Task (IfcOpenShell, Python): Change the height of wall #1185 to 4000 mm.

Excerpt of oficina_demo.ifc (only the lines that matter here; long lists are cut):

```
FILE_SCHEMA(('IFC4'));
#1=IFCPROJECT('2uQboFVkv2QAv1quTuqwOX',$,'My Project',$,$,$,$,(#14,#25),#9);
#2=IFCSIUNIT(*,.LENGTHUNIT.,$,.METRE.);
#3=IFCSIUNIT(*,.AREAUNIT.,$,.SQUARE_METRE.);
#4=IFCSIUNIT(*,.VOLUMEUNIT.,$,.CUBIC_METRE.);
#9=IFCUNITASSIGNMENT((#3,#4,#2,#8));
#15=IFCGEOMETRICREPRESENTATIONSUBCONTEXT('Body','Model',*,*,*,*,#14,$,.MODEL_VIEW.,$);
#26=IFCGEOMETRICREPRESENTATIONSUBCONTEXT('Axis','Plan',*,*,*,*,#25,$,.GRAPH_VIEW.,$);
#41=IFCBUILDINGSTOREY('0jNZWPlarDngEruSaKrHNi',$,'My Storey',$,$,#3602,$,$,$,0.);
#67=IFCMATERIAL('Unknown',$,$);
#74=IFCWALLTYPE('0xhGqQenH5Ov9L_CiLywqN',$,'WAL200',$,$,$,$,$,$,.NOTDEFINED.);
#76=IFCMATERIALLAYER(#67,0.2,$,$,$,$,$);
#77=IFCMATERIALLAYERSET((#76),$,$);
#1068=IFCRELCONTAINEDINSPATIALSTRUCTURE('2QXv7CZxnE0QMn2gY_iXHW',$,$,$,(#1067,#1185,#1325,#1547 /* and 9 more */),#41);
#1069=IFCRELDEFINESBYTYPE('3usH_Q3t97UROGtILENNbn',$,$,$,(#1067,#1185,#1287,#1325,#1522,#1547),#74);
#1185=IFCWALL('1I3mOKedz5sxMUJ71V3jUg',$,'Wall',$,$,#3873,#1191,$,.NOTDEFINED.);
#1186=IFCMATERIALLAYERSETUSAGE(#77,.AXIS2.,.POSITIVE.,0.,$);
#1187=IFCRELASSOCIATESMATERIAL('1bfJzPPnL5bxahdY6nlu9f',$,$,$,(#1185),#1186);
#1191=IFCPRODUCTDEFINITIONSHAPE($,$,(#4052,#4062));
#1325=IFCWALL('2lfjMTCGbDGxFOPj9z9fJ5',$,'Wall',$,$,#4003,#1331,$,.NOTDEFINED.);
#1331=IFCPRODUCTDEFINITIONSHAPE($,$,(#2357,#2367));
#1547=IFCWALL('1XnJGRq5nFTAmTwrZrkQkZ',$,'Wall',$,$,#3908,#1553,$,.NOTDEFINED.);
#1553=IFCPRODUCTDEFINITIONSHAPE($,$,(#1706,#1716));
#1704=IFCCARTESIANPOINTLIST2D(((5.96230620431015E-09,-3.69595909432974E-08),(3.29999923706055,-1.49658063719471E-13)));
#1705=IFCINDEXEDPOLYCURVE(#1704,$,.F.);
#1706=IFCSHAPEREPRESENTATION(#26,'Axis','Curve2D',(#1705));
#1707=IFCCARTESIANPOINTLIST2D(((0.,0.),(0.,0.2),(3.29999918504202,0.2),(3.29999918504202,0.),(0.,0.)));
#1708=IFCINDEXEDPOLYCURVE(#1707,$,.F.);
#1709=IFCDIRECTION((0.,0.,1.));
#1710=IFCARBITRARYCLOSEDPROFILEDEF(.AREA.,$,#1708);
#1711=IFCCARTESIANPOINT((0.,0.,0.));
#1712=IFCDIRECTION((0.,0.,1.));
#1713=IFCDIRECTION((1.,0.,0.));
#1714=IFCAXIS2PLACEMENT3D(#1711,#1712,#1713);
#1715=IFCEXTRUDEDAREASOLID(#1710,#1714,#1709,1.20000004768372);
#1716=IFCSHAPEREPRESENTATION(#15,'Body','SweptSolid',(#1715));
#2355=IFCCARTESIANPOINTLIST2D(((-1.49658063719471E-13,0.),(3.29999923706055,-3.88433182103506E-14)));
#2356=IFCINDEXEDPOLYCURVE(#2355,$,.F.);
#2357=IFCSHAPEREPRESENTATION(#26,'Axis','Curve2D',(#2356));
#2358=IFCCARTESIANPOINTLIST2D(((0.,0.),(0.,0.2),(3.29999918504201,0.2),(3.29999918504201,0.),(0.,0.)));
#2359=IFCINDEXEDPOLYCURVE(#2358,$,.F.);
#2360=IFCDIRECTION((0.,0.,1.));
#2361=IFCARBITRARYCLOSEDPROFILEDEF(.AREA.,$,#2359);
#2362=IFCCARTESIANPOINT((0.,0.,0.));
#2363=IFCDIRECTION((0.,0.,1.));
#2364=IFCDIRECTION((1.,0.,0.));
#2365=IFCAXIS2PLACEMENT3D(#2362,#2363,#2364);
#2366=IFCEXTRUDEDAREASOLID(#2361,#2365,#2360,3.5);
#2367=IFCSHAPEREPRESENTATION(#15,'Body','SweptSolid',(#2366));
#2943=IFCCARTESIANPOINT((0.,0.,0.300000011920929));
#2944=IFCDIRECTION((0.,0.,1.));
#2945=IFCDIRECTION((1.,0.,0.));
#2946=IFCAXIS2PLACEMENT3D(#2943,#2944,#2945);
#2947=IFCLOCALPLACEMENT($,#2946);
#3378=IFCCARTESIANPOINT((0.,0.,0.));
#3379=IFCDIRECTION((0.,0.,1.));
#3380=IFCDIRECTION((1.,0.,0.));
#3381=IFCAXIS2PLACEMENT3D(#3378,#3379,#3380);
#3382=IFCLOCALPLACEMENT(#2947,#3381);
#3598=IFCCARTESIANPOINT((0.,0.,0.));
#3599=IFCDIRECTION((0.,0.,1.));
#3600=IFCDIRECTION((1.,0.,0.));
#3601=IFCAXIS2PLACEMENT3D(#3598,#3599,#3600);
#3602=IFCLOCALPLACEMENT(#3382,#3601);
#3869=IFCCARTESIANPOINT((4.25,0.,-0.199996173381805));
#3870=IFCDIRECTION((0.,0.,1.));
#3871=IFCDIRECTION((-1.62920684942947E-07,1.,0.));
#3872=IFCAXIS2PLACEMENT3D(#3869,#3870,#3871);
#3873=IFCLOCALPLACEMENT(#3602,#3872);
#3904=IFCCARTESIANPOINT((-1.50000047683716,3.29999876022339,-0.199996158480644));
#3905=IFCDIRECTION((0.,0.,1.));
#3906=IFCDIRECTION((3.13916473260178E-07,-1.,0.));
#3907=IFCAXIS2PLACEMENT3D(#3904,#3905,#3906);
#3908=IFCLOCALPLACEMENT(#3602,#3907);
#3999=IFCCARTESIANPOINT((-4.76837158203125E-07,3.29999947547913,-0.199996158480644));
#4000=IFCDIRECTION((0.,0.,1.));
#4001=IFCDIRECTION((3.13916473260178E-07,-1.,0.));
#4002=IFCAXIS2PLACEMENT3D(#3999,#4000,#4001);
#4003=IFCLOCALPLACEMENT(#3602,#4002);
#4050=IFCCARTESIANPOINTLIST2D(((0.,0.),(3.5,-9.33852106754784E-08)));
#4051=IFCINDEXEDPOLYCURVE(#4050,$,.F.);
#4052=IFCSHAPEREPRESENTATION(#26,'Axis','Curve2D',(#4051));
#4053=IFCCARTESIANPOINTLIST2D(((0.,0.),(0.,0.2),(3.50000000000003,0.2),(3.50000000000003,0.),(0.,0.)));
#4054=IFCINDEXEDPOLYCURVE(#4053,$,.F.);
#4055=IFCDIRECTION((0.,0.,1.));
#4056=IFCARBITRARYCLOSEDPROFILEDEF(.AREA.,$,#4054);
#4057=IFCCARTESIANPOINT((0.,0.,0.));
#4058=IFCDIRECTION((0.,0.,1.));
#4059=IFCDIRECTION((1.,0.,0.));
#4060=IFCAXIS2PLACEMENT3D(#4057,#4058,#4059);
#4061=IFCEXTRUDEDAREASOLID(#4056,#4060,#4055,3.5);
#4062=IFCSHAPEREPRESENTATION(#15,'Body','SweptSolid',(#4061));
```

```python
import ifcopenshell
import ifcopenshell.geom
import ifcopenshell.util.representation
import ifcopenshell.util.shape

model = ifcopenshell.open("oficina_demo.ifc")
settings = ifcopenshell.geom.settings()


def volume(element):
    """Net volume in cubic metres, openings subtracted."""
    shape = ifcopenshell.geom.create_shape(settings, element)
    return ifcopenshell.util.shape.get_volume(shape.geometry)


wall = model.by_guid("1I3mOKedz5sxMUJ71V3jUg")
before = volume(wall)

body = ifcopenshell.util.representation.get_representation(wall, "Model", "Body")
solid = body.Items[0]
old_height = solid.Depth
solid.Depth = 4.0
after = volume(wall)

print(f"height {old_height:g} -> {solid.Depth:g}, volume {before:.3f} -> {after:.3f} m3")

model.write("oficina_demo_updated.ifc")
```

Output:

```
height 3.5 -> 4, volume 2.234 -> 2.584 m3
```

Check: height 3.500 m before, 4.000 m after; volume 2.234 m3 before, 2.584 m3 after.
